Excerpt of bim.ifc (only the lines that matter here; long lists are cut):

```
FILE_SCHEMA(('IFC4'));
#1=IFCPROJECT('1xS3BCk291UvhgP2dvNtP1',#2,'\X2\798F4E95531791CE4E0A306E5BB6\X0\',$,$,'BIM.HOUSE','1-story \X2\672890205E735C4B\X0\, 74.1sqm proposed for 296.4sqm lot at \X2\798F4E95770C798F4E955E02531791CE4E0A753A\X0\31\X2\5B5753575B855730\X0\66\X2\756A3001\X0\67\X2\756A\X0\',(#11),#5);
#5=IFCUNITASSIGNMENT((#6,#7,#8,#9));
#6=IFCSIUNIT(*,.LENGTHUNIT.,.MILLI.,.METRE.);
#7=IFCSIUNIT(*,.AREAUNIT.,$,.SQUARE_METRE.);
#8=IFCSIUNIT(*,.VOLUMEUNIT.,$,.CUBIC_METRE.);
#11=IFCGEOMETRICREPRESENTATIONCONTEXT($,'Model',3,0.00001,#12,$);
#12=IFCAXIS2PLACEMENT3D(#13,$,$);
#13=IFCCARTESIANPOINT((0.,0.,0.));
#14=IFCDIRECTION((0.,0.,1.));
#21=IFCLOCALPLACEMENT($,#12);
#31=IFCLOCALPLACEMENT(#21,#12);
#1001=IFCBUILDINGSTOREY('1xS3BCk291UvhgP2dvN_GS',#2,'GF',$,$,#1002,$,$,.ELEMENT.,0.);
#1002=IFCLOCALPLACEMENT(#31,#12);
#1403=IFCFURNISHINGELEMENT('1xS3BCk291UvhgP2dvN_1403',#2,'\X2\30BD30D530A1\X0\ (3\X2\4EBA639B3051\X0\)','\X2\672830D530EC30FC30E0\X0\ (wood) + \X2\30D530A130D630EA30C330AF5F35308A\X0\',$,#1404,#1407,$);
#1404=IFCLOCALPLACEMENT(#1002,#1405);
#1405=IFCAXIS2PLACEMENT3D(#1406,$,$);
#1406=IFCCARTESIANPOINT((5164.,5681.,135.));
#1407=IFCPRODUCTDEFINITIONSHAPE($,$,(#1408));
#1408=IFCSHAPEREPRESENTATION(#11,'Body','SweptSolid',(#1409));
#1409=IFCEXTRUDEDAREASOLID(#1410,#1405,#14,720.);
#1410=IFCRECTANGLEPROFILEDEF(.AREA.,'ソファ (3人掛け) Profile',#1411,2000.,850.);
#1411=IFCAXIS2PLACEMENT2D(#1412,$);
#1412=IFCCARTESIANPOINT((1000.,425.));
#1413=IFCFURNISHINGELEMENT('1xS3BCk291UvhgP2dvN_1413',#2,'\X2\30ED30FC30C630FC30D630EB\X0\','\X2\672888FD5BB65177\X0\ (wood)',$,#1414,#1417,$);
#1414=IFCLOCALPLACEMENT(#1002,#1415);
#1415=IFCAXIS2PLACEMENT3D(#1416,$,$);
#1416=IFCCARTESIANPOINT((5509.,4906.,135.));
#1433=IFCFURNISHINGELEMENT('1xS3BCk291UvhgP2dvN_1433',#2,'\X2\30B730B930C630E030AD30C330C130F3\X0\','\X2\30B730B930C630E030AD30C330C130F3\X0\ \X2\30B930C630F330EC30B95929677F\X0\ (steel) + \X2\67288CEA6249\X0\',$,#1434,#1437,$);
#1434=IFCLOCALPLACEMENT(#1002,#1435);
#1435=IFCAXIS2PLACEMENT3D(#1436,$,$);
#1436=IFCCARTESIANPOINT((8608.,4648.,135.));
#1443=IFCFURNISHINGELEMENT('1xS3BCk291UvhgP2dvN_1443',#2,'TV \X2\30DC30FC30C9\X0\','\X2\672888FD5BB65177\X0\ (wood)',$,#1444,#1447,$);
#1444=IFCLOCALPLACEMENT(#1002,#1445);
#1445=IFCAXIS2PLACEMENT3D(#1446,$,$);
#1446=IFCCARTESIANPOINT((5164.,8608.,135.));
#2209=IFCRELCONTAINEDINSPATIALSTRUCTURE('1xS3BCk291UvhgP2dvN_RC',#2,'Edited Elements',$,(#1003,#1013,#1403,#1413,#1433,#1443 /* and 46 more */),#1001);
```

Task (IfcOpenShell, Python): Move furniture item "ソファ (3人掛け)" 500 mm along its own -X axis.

```python
import ifcopenshell
import ifcopenshell.api.geometry
import ifcopenshell.util.placement
import ifcopenshell.util.unit

model = ifcopenshell.open("bim.ifc")
unit_scale = ifcopenshell.util.unit.calculate_unit_scale(model)

item = model.by_guid("1xS3BCk291UvhgP2dvN_1403")
matrix = ifcopenshell.util.placement.get_local_placement(item.ObjectPlacement)
matrix[:3, 3] -= matrix[:3, 0] * 0.5 / unit_scale
ifcopenshell.api.geometry.edit_object_placement(model, product=item, matrix=matrix, is_si=False)

print(ifcopenshell.util.placement.get_local_placement(item.ObjectPlacement).round(3) + 0.0)

model.write("bim_rev.ifc")
```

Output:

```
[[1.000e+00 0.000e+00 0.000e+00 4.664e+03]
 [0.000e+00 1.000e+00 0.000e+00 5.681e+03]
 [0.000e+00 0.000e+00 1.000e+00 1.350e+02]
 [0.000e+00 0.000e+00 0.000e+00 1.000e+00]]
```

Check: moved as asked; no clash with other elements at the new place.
